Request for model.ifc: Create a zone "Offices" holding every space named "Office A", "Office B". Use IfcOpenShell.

First a look at what the model holds.

```python
import ifcopenshell

model = ifcopenshell.open("model.ifc")
print(model.schema)
seen = {}
for space in model.by_type("IfcSpace"):
    seen[space.LongName] = seen.get(space.LongName, 0) + 1
for name, count in sorted(seen.items(), key=str):
    print(count, "x", name)
print("zones:", [z.Name for z in model.by_type("IfcZone")][:20])
```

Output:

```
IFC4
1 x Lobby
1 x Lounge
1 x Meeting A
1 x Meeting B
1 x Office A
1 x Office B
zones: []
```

```python
import ifcopenshell
import ifcopenshell.api.group
import ifcopenshell.api.root

model = ifcopenshell.open("model.ifc")

names = {"Office A", "Office B"}
spaces = [s for s in model.by_type("IfcSpace") if s.LongName in names]

zone = ifcopenshell.api.root.create_entity(model, ifc_class="IfcZone", name="Offices")
ifcopenshell.api.group.assign_group(model, products=spaces, group=zone)
print(len(spaces), "spaces in", zone.Name)

model.write("model-out.ifc")
```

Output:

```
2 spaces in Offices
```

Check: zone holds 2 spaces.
